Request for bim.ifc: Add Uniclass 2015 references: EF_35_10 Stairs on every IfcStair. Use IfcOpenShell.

First a look at what the model holds.

```python
import ifcopenshell

model = ifcopenshell.open("bim.ifc")
print(model.schema)
print("classifications:", [c.Name for c in model.by_type("IfcClassification")])
for ifc_class in ("IfcDoor", "IfcRoof", "IfcStair", "IfcWall", "IfcWindow"):
    print(ifc_class, len(model.by_type(ifc_class)))
```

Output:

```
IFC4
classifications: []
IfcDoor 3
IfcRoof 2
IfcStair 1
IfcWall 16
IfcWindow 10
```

```python
import ifcopenshell
import ifcopenshell.api.classification

model = ifcopenshell.open("bim.ifc")

system = ifcopenshell.api.classification.add_classification(model, classification="Uniclass 2015")

codes = {
    "IfcStair": ("EF_35_10", "Stairs"),
}
for ifc_class, (code, name) in codes.items():
    products = model.by_type(ifc_class)
    ifcopenshell.api.classification.add_reference(
        model, products=products, classification=system, identification=code, name=name
    )
    print(code, len(products))

model.write("bim-out.ifc")
```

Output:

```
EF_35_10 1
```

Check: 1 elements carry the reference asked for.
